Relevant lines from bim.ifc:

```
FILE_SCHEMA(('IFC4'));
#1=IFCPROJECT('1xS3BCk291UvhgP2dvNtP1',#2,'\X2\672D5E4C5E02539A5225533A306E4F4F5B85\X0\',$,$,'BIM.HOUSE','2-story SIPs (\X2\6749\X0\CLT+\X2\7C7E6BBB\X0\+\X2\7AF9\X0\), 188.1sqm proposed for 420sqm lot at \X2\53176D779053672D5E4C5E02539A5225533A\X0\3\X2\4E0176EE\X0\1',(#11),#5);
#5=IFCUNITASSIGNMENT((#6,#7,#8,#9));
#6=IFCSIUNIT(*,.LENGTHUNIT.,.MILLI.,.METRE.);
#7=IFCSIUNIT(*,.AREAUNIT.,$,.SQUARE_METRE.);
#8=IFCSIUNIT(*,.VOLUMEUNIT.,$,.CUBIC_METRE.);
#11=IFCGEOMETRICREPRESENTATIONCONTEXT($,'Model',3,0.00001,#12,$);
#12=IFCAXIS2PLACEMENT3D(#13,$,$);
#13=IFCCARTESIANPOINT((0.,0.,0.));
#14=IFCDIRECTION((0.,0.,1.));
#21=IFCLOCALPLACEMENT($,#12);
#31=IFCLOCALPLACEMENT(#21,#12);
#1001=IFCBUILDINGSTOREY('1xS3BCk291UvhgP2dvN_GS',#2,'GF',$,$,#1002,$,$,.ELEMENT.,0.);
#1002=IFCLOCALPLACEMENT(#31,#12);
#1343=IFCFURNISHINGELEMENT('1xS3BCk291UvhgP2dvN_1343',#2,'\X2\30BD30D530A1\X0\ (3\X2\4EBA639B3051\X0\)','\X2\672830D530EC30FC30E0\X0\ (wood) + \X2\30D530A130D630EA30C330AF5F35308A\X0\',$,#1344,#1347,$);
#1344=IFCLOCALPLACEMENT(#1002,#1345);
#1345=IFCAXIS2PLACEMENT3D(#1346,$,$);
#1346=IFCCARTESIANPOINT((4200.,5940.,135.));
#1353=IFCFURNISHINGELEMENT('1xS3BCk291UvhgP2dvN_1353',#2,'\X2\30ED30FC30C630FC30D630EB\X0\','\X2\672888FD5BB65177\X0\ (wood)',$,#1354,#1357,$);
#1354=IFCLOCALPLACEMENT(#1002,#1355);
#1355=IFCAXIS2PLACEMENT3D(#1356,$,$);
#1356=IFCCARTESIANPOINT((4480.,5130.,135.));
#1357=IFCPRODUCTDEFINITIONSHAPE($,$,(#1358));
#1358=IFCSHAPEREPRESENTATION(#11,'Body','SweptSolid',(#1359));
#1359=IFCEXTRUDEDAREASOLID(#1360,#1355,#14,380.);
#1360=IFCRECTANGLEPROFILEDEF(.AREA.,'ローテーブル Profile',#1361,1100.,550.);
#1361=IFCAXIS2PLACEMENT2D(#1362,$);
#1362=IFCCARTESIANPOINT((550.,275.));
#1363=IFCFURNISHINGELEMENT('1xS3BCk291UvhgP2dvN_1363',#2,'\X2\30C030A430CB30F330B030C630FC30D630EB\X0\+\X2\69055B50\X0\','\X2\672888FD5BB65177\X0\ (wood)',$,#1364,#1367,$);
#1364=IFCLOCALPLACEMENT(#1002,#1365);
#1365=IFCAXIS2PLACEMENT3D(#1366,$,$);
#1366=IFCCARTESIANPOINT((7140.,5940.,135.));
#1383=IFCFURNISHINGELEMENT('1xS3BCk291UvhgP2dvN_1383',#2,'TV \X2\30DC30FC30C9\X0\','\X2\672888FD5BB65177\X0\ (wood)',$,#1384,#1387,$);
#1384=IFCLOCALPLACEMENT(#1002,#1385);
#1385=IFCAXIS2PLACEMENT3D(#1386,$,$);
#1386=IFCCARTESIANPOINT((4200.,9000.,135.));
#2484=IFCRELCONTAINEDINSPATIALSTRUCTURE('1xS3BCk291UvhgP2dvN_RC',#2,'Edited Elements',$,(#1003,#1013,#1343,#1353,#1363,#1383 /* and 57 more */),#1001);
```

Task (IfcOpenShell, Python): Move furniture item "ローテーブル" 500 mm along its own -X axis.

```python
import ifcopenshell
import ifcopenshell.api.geometry
import ifcopenshell.util.placement
import ifcopenshell.util.unit

model = ifcopenshell.open("bim.ifc")
unit_scale = ifcopenshell.util.unit.calculate_unit_scale(model)

item = model.by_guid("1xS3BCk291UvhgP2dvN_1353")
matrix = ifcopenshell.util.placement.get_local_placement(item.ObjectPlacement)
matrix[:3, 3] -= matrix[:3, 0] * 0.5 / unit_scale
ifcopenshell.api.geometry.edit_object_placement(model, product=item, matrix=matrix, is_si=False)

print(ifcopenshell.util.placement.get_local_placement(item.ObjectPlacement).round(3) + 0.0)

model.write("bim_updated.ifc")
```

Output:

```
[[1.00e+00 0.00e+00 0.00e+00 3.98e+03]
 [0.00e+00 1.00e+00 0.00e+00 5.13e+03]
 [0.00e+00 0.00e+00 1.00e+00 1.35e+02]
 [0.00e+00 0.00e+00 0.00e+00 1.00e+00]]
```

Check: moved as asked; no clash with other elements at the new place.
